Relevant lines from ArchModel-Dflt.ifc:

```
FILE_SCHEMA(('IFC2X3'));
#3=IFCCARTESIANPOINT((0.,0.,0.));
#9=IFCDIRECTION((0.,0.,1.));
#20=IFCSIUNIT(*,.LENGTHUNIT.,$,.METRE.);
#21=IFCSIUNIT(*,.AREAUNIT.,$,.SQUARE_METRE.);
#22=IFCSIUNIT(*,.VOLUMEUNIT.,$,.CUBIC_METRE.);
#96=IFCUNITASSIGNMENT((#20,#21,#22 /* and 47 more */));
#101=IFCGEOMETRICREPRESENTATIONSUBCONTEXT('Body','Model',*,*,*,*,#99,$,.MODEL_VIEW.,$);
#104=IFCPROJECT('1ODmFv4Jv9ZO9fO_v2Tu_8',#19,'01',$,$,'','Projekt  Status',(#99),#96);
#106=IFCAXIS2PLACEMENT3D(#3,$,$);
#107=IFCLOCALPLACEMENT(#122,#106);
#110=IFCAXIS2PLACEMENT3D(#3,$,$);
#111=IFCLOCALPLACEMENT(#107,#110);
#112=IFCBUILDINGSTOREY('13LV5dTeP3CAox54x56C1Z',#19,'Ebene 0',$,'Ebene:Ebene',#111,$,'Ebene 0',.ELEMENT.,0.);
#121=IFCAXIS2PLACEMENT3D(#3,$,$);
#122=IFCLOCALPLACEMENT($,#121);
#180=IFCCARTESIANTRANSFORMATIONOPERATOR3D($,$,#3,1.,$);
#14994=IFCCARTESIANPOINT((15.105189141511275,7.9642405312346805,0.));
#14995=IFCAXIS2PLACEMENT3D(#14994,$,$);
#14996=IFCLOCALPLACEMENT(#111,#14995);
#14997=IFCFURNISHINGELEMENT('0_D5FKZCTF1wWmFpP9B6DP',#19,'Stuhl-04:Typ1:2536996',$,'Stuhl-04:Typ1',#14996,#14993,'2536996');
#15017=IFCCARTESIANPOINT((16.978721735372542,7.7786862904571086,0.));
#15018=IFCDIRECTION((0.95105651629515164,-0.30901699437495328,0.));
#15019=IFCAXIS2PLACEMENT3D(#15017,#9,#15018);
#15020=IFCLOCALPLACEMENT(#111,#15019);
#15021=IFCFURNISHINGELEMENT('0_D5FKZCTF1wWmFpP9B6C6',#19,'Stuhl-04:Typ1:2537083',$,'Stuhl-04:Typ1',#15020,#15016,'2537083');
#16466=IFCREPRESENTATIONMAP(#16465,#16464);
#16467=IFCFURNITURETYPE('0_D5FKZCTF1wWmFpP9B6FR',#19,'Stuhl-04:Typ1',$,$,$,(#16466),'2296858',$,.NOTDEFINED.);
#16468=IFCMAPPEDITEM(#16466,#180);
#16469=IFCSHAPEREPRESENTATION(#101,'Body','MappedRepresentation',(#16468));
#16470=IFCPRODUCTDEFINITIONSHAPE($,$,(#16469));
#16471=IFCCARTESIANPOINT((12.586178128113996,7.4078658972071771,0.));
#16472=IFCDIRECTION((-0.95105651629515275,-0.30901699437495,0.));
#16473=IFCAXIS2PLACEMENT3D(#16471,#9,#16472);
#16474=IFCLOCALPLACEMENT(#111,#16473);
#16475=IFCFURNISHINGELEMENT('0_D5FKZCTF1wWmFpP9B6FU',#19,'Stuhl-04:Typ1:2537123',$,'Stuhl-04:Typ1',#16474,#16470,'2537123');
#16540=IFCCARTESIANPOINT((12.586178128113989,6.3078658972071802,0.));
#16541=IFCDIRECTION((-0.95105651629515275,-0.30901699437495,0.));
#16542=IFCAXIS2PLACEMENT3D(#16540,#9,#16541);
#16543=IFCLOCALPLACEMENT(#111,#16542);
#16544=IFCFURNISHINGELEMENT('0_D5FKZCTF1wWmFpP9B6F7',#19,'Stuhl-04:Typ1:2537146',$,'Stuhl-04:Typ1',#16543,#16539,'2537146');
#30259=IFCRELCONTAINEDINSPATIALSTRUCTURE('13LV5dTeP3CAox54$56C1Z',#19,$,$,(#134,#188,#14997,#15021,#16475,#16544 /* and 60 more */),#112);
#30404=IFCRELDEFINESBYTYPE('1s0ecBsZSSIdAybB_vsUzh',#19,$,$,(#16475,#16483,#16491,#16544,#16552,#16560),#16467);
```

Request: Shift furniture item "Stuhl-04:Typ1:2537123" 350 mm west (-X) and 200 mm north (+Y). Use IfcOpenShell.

```python
import ifcopenshell
import ifcopenshell.api.geometry
import ifcopenshell.util.placement
import ifcopenshell.util.unit

model = ifcopenshell.open("ArchModel-Dflt.ifc")
unit_scale = ifcopenshell.util.unit.calculate_unit_scale(model)

item = model.by_guid("0_D5FKZCTF1wWmFpP9B6FU")
matrix = ifcopenshell.util.placement.get_local_placement(item.ObjectPlacement)
matrix[0, 3] -= 0.35 / unit_scale
matrix[1, 3] += 0.2 / unit_scale
ifcopenshell.api.geometry.edit_object_placement(model, product=item, matrix=matrix, is_si=False)

print(ifcopenshell.util.placement.get_local_placement(item.ObjectPlacement).round(3) + 0.0)

model.write("ArchModel-Dflt_edited.ifc")
```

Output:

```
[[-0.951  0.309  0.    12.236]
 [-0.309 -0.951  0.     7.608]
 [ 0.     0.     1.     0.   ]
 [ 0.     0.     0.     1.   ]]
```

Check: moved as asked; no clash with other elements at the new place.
